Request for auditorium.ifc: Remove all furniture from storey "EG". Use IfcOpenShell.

First a look at what the model holds.

```python
import ifcopenshell
import ifcopenshell.util.element

model = ifcopenshell.open("auditorium.ifc")
print(model.schema)
storey = next(s for s in model.by_type("IfcBuildingStorey") if s.Name == "EG")
furniture = [e for e in ifcopenshell.util.element.get_decomposition(storey) if e.is_a("IfcFurnishingElement")]
seen = {}
for e in furniture:
    element_type = ifcopenshell.util.element.get_type(e)
    name = element_type.Name if element_type not in (None, e) else None
    seen[name] = seen.get(name, 0) + 1
for name, count in sorted(seen.items(), key=str):
    print(count, "x", name)
```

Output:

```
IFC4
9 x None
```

```python
import ifcopenshell
import ifcopenshell.api.root
import ifcopenshell.util.element

model = ifcopenshell.open("auditorium.ifc")

storey = next(s for s in model.by_type("IfcBuildingStorey") if s.Name == "EG")
furniture = [e for e in ifcopenshell.util.element.get_decomposition(storey) if e.is_a("IfcFurnishingElement")]

for e in furniture:
    ifcopenshell.api.root.remove_product(model, product=e)
print(len(furniture), "removed")

model.write("auditorium_v2.ifc")
```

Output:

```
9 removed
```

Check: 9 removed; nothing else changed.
